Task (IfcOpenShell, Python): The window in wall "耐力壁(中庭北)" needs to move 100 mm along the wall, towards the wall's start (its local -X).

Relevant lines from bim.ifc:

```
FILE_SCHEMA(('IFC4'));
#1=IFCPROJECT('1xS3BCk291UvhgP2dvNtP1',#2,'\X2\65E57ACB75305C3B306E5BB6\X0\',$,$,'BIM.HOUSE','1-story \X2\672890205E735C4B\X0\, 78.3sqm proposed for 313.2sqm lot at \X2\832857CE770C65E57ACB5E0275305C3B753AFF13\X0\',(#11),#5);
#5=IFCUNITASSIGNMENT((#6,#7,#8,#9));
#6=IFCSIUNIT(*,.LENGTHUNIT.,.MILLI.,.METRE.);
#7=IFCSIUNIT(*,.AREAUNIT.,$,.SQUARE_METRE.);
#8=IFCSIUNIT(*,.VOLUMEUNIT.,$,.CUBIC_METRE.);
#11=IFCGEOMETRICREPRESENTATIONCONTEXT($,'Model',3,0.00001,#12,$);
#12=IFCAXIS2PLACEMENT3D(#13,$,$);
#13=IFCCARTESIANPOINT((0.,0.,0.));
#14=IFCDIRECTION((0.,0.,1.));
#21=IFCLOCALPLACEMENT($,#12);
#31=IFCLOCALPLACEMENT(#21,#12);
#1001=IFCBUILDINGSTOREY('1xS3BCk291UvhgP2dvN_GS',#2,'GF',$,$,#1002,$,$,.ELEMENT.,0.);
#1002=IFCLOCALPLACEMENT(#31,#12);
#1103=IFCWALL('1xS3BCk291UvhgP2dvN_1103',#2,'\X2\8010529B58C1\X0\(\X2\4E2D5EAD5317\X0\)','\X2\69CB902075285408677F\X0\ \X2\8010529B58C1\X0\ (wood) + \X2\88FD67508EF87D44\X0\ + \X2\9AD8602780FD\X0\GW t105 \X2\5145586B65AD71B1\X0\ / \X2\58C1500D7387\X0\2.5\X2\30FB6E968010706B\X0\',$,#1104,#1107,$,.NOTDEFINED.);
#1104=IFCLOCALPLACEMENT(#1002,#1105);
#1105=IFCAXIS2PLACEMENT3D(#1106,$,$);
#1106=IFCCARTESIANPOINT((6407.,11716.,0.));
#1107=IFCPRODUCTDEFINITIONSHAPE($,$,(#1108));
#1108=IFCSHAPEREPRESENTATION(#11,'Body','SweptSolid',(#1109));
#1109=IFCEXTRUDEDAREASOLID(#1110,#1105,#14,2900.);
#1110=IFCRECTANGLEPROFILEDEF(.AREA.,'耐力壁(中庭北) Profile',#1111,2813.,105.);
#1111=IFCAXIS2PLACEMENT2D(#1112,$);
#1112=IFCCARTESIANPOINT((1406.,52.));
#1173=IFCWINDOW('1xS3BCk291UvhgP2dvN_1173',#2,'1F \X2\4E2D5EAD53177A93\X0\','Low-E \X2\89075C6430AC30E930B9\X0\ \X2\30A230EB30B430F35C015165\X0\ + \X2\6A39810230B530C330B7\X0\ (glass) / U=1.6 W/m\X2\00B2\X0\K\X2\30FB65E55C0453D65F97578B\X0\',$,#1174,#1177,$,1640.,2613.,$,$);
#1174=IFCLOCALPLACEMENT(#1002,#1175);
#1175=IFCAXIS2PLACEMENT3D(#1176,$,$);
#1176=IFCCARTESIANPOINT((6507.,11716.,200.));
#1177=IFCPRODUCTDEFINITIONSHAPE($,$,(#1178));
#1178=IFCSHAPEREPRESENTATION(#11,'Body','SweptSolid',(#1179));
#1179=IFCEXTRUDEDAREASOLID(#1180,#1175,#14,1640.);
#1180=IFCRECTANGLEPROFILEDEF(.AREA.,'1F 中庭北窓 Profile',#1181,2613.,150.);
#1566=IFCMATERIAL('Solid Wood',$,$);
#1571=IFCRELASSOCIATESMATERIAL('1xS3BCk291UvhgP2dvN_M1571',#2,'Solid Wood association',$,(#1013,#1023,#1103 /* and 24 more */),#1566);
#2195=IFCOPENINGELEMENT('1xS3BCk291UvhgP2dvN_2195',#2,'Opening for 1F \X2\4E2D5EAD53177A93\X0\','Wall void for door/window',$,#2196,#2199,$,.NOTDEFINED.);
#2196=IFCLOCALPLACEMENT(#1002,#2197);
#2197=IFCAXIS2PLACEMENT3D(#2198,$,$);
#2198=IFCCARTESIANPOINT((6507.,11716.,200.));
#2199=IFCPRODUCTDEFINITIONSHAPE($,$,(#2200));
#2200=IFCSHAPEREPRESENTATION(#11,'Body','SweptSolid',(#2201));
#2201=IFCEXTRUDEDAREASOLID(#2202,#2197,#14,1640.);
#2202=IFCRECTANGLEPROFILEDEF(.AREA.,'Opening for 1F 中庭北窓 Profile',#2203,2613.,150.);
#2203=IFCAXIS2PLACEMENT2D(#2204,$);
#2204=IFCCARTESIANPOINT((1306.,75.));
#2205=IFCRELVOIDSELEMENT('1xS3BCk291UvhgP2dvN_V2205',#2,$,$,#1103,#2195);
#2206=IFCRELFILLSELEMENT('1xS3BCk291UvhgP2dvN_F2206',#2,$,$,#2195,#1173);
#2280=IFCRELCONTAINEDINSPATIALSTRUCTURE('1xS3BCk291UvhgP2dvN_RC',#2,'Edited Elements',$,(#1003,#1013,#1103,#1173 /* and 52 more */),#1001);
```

```python
import ifcopenshell
import ifcopenshell.api.geometry
import ifcopenshell.util.placement
import ifcopenshell.util.unit

model = ifcopenshell.open("bim.ifc")
unit_scale = ifcopenshell.util.unit.calculate_unit_scale(model)

window = model.by_guid("1xS3BCk291UvhgP2dvN_1173")
opening = window.FillsVoids[0].RelatingOpeningElement
wall = opening.VoidsElements[0].RelatingBuildingElement

wall_matrix = ifcopenshell.util.placement.get_local_placement(wall.ObjectPlacement)
shift = wall_matrix[:3, 0] * -0.1 / unit_scale
before = ifcopenshell.util.placement.get_local_placement(window.ObjectPlacement)[:3, 3].copy()

# The window is not placed relative to its opening, so move both.
for product in (opening, window):
    matrix = ifcopenshell.util.placement.get_local_placement(product.ObjectPlacement)
    matrix[:3, 3] += shift
    ifcopenshell.api.geometry.edit_object_placement(model, product=product, matrix=matrix, is_si=False)

after = ifcopenshell.util.placement.get_local_placement(window.ObjectPlacement)[:3, 3]
print("window moved by", (after - before).round(3) + 0.0)

model.write("bim_rev.ifc")
```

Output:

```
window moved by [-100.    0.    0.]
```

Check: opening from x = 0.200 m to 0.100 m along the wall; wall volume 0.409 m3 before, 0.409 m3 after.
